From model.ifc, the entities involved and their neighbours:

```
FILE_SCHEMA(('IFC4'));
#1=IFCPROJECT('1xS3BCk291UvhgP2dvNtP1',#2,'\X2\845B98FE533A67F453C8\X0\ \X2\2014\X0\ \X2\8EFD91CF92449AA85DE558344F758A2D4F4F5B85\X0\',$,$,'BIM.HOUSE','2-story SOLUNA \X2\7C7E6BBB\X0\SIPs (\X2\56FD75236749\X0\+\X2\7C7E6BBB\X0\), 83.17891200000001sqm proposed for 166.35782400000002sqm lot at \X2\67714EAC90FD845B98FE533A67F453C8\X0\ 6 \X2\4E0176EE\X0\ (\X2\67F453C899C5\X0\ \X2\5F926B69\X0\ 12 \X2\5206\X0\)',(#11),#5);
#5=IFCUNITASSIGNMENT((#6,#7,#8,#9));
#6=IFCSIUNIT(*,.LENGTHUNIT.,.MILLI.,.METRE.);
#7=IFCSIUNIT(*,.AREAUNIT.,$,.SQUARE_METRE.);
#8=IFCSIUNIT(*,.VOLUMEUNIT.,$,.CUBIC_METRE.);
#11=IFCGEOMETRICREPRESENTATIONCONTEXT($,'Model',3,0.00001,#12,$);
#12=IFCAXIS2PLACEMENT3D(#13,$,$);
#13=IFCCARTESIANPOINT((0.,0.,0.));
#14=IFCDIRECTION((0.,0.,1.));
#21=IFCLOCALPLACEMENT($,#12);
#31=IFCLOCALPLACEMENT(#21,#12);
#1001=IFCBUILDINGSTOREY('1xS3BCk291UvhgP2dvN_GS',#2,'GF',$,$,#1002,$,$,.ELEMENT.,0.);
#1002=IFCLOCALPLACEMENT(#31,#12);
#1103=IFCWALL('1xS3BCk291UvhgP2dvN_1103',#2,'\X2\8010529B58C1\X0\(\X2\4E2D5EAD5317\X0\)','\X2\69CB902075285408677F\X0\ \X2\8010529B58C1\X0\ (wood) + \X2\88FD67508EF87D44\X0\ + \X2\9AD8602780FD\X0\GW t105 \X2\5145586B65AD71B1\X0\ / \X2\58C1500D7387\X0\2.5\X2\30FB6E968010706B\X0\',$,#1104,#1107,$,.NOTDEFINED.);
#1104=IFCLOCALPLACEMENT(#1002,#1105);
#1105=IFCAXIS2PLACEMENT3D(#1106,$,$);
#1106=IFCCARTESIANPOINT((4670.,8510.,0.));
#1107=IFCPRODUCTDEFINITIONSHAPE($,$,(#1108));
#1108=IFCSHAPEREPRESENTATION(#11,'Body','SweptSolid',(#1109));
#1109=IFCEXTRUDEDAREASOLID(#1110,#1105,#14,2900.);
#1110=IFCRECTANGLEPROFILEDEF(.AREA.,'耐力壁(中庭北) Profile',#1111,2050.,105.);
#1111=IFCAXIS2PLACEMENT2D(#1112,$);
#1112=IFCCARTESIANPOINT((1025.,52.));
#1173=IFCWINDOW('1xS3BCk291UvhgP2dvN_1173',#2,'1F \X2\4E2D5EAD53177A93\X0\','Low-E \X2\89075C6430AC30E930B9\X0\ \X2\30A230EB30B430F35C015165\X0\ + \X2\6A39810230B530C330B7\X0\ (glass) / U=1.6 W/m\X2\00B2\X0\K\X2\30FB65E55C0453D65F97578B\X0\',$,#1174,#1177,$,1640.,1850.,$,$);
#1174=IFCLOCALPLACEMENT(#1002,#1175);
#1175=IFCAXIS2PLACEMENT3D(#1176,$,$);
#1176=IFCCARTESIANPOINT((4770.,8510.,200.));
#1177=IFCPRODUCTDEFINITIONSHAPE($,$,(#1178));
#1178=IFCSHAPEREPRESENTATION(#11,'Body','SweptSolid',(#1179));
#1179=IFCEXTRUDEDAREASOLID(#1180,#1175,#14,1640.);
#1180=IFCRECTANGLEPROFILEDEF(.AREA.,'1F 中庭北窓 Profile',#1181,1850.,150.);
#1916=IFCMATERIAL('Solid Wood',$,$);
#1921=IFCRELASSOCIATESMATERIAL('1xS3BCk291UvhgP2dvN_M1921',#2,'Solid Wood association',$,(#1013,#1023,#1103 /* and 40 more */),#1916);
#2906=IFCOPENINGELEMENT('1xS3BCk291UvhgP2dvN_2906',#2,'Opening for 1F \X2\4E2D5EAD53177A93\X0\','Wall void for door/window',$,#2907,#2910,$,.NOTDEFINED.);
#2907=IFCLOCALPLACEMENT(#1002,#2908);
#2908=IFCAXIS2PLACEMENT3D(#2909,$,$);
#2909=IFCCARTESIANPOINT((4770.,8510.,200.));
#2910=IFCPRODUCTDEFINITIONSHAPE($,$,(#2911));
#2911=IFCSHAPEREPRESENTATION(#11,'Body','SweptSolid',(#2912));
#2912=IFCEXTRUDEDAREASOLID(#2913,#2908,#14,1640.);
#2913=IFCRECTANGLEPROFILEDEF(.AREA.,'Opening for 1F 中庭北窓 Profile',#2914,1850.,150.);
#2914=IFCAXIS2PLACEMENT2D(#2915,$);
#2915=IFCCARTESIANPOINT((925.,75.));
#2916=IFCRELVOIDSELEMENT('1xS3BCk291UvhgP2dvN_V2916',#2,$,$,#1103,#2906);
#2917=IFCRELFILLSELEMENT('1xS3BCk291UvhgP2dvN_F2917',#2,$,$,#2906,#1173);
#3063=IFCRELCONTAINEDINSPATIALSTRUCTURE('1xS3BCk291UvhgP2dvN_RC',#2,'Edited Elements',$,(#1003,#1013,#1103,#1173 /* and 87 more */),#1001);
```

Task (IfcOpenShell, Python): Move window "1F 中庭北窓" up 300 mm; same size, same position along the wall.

```python
import numpy as np
import ifcopenshell
import ifcopenshell.api.geometry
import ifcopenshell.util.placement
import ifcopenshell.util.unit

model = ifcopenshell.open("model.ifc")
unit_scale = ifcopenshell.util.unit.calculate_unit_scale(model)

window = model.by_guid("1xS3BCk291UvhgP2dvN_1173")
opening = window.FillsVoids[0].RelatingOpeningElement
dz = 0.3 / unit_scale

shift = np.array([0.0, 0.0, dz])
# The window is not placed relative to its opening, so move both.
for product in (opening, window):
    matrix = ifcopenshell.util.placement.get_local_placement(product.ObjectPlacement)
    matrix[:3, 3] += shift
    ifcopenshell.api.geometry.edit_object_placement(model, product=product, matrix=matrix, is_si=False)

print(f"moved by {dz * unit_scale:+.3f} m")

model.write("model-out.ifc")
```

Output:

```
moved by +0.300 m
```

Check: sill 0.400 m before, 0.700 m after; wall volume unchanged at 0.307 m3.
